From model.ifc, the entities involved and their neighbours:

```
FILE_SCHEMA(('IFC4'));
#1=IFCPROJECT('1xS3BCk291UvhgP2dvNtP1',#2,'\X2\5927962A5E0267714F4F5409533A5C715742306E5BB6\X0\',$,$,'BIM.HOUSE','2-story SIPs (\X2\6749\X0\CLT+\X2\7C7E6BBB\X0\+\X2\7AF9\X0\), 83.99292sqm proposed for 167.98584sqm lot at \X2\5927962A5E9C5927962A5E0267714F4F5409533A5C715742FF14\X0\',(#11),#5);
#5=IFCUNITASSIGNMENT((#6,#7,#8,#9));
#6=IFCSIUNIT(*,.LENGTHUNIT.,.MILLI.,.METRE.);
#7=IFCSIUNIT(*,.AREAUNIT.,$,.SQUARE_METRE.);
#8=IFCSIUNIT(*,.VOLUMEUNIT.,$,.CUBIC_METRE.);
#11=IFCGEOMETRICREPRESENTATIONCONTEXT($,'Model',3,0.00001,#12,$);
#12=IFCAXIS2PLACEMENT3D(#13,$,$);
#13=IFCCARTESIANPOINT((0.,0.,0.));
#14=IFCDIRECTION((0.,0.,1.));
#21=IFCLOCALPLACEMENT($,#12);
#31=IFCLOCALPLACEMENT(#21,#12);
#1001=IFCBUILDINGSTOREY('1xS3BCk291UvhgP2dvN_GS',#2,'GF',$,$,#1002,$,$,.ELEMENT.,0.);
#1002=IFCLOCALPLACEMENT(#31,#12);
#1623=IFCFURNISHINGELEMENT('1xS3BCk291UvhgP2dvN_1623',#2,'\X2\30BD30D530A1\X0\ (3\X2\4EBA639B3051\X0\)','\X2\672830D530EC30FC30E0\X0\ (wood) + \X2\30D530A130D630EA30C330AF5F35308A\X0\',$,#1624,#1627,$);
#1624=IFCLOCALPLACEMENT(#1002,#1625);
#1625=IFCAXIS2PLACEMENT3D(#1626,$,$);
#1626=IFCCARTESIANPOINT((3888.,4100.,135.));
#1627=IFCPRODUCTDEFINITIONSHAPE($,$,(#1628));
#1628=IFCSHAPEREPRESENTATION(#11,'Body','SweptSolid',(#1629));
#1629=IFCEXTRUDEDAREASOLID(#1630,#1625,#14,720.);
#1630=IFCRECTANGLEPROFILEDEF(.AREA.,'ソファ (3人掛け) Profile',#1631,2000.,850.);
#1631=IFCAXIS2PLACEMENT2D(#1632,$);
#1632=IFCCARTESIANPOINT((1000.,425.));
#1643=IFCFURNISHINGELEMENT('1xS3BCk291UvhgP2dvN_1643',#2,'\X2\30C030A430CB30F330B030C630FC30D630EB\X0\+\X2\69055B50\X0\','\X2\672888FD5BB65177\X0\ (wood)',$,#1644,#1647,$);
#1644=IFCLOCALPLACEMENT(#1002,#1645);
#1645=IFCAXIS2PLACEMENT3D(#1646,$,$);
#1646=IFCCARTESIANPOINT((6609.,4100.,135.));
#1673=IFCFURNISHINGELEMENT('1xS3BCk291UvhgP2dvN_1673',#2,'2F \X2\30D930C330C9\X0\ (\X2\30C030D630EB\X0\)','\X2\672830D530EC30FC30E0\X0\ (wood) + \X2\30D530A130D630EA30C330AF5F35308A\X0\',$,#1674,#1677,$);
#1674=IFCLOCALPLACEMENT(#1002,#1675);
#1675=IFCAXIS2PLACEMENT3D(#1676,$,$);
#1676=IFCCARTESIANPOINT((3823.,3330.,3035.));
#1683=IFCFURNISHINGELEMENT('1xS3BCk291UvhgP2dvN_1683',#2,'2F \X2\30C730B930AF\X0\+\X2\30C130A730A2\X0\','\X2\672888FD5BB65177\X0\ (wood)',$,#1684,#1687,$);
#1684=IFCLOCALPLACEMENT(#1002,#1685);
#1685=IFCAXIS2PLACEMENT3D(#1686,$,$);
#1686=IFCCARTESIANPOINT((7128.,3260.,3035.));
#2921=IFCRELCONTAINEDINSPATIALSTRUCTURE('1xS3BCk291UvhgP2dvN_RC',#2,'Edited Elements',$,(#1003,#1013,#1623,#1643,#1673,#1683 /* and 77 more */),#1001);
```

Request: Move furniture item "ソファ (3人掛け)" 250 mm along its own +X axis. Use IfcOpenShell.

```python
import ifcopenshell
import ifcopenshell.api.geometry
import ifcopenshell.util.placement
import ifcopenshell.util.unit

model = ifcopenshell.open("model.ifc")
unit_scale = ifcopenshell.util.unit.calculate_unit_scale(model)

item = model.by_guid("1xS3BCk291UvhgP2dvN_1623")
matrix = ifcopenshell.util.placement.get_local_placement(item.ObjectPlacement)
matrix[:3, 3] += matrix[:3, 0] * 0.25 / unit_scale
ifcopenshell.api.geometry.edit_object_placement(model, product=item, matrix=matrix, is_si=False)

print(ifcopenshell.util.placement.get_local_placement(item.ObjectPlacement).round(3) + 0.0)

model.write("model-out.ifc")
```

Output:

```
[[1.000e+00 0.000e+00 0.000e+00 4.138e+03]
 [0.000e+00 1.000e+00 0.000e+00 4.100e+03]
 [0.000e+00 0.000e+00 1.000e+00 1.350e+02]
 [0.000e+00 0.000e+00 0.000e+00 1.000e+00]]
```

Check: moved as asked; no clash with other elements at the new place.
